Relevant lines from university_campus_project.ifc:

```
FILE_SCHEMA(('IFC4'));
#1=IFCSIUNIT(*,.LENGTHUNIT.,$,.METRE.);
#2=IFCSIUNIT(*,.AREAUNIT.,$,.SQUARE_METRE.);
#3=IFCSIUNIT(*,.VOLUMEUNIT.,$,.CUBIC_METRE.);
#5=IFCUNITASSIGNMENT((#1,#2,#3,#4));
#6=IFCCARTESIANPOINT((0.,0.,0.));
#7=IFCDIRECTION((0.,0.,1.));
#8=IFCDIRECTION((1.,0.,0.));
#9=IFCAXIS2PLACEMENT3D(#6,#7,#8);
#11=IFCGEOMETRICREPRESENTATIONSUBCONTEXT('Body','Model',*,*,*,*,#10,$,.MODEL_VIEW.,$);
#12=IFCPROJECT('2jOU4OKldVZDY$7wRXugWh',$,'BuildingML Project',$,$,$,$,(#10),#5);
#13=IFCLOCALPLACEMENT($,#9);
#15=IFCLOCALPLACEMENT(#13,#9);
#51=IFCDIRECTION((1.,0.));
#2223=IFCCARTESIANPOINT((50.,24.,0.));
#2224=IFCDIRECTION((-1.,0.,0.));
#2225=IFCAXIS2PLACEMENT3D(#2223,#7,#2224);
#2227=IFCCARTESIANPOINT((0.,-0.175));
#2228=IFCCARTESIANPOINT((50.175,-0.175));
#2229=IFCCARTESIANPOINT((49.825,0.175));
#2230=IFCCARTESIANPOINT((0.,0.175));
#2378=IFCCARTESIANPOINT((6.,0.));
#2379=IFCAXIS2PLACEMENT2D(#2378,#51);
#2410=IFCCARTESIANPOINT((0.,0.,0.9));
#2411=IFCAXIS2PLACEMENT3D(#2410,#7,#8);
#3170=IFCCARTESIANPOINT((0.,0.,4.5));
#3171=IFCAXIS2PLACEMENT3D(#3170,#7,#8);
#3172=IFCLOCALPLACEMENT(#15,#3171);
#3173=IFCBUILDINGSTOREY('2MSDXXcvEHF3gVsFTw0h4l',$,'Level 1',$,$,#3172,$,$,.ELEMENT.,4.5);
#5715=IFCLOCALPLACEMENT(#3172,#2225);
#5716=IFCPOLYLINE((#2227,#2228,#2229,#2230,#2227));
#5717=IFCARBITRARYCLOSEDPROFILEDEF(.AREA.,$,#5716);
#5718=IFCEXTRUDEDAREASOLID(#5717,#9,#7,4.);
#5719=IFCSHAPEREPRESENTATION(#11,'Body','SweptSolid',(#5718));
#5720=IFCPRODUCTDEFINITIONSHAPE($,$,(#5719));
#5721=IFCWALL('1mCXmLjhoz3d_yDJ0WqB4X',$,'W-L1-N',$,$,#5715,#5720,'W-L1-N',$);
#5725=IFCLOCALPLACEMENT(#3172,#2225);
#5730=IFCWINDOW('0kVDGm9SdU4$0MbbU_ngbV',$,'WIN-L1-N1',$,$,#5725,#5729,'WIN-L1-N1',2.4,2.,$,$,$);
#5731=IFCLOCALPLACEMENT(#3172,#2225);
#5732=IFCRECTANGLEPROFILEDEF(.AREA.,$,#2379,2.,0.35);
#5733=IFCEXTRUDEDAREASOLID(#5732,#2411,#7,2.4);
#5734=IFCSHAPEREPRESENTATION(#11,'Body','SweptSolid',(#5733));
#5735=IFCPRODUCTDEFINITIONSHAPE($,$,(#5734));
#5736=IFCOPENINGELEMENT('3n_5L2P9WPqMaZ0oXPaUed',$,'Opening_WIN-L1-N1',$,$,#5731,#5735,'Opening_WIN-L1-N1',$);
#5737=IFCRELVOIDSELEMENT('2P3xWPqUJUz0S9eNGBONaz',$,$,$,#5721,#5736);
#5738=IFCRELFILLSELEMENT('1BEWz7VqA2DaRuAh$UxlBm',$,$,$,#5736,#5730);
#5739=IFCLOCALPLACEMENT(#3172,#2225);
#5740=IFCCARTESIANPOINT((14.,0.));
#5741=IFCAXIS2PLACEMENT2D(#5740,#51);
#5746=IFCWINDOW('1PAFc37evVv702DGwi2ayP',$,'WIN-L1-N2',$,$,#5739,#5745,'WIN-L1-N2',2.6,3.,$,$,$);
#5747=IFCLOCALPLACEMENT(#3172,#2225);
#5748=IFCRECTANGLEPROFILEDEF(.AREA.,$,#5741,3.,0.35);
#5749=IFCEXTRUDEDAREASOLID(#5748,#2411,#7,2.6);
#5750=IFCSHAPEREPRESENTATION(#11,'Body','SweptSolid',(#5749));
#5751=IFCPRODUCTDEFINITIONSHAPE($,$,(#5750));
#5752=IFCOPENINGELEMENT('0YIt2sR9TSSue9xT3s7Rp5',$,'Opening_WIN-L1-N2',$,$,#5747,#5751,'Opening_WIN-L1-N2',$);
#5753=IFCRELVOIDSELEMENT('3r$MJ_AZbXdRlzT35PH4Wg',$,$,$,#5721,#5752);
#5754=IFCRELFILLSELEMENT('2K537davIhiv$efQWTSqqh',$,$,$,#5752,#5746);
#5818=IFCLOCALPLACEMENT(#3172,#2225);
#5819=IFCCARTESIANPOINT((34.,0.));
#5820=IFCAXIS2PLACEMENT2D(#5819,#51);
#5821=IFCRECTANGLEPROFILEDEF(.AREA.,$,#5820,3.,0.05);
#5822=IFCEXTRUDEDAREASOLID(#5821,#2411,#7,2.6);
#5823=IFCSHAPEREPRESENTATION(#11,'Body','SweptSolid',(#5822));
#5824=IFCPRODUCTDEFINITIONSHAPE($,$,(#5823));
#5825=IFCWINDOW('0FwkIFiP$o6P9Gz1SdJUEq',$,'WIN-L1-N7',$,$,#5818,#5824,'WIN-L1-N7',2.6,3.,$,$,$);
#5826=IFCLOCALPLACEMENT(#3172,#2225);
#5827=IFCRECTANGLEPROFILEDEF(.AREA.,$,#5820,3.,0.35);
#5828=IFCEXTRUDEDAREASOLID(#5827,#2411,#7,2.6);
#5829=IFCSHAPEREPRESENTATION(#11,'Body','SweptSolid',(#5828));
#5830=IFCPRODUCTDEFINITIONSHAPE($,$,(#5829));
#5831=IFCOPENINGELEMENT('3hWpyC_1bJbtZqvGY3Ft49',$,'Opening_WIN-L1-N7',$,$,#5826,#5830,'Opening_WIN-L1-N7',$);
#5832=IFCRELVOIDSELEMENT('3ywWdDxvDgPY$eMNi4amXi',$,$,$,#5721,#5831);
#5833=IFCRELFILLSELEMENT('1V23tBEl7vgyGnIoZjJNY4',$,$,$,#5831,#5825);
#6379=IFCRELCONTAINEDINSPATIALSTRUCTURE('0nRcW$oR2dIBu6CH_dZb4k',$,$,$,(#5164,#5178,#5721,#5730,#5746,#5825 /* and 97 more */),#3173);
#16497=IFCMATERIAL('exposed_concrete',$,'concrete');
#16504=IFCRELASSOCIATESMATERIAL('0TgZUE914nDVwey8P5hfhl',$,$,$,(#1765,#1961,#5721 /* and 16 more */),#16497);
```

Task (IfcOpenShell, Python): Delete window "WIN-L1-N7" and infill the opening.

```python
import ifcopenshell
import ifcopenshell.api.feature
import ifcopenshell.api.root
import ifcopenshell.geom
import ifcopenshell.util.shape

model = ifcopenshell.open("university_campus_project.ifc")
settings = ifcopenshell.geom.settings()


def volume(element):
    """Net volume in cubic metres, openings subtracted."""
    shape = ifcopenshell.geom.create_shape(settings, element)
    return ifcopenshell.util.shape.get_volume(shape.geometry)


window = model.by_id(5825)
opening = window.FillsVoids[0].RelatingOpeningElement
wall = opening.VoidsElements[0].RelatingBuildingElement
before = volume(wall)

ifcopenshell.api.root.remove_product(model, product=window)
ifcopenshell.api.feature.remove_feature(model, feature=opening)

after = volume(wall)

print(f"wall volume {before:.3f} -> {after:.3f} m3")

model.write("university_campus_project_v2.ifc")
```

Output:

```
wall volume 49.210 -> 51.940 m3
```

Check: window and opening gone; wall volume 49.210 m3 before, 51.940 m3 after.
